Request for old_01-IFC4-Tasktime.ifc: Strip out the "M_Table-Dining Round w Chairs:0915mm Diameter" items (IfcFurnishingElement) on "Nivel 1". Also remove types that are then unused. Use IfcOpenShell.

First a look at what the model holds.

```python
import ifcopenshell
import ifcopenshell.util.element

model = ifcopenshell.open("old_01-IFC4-Tasktime.ifc")
print(model.schema)
storey = next(s for s in model.by_type("IfcBuildingStorey") if s.Name == "Nivel 1")
furniture = [e for e in ifcopenshell.util.element.get_decomposition(storey) if e.is_a("IfcFurnishingElement")]
seen = {}
for e in furniture:
    element_type = ifcopenshell.util.element.get_type(e)
    name = element_type.Name if element_type not in (None, e) else None
    seen[name] = seen.get(name, 0) + 1
for name, count in sorted(seen.items(), key=str):
    print(count, "x", name)
```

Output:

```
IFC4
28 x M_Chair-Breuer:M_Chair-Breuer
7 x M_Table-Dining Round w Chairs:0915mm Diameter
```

```python
import ifcopenshell
import ifcopenshell.api.root
import ifcopenshell.util.element

model = ifcopenshell.open("old_01-IFC4-Tasktime.ifc")

storey = next(s for s in model.by_type("IfcBuildingStorey") if s.Name == "Nivel 1")
furniture = [e for e in ifcopenshell.util.element.get_decomposition(storey) if e.is_a("IfcFurnishingElement")]
targets = [e for e in furniture if (t := ifcopenshell.util.element.get_type(e)) not in (None, e) and t.Name == "M_Table-Dining Round w Chairs:0915mm Diameter"]
types = {ifcopenshell.util.element.get_type(e) for e in targets} - {None, *targets}

for e in targets:
    ifcopenshell.api.root.remove_product(model, product=e)
print(len(targets), "removed")

unused = [t for t in types if not ifcopenshell.util.element.get_types(t)]
for t in unused:
    ifcopenshell.api.root.remove_product(model, product=t)
print(len(unused), "unused types removed")

model.write("old_01-IFC4-Tasktime_edited.ifc")
```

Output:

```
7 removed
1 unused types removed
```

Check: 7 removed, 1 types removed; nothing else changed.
